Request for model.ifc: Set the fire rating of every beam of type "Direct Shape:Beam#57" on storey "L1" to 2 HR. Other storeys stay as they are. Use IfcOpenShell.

First a look at what the model holds.

```python
import ifcopenshell
import ifcopenshell.util.element

model = ifcopenshell.open("model.ifc")
print(model.schema)
storey = next(s for s in model.by_type("IfcBuildingStorey") if s.Name == "L1")
beams = [e for e in ifcopenshell.util.element.get_decomposition(storey) if e.is_a("IfcBeam")]
seen = {}
for e in beams:
    element_type = ifcopenshell.util.element.get_type(e)
    key = (element_type.Name if element_type != e and element_type else None, ifcopenshell.util.element.get_pset(e, "Pset_BeamCommon", "FireRating"))
    seen[key] = seen.get(key, 0) + 1
for (name, value), count in sorted(seen.items(), key=str):
    print(count, "x", name, "|", value)
```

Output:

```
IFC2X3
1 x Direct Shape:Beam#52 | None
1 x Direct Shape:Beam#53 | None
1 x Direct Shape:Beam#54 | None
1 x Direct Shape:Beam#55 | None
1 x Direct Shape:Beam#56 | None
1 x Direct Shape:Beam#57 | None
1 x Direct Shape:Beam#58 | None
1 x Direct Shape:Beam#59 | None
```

```python
import ifcopenshell
import ifcopenshell.api.pset
import ifcopenshell.util.element

model = ifcopenshell.open("model.ifc")

storey = next(s for s in model.by_type("IfcBuildingStorey") if s.Name == "L1")
beams = [e for e in ifcopenshell.util.element.get_decomposition(storey) if e.is_a("IfcBeam")]

count = 0
for e in beams:
    element_type = ifcopenshell.util.element.get_type(e)
    if element_type in (None, e) or element_type.Name != "Direct Shape:Beam#57":
        continue
    # add_pset returns the element's existing set when there is one.
    pset = ifcopenshell.api.pset.add_pset(model, product=e, name="Pset_BeamCommon")
    ifcopenshell.api.pset.edit_pset(model, pset=pset, properties={"FireRating": "2 HR"})
    count += 1

print(count, "beams updated")

model.write("model-out.ifc")
```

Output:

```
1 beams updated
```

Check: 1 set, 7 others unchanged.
